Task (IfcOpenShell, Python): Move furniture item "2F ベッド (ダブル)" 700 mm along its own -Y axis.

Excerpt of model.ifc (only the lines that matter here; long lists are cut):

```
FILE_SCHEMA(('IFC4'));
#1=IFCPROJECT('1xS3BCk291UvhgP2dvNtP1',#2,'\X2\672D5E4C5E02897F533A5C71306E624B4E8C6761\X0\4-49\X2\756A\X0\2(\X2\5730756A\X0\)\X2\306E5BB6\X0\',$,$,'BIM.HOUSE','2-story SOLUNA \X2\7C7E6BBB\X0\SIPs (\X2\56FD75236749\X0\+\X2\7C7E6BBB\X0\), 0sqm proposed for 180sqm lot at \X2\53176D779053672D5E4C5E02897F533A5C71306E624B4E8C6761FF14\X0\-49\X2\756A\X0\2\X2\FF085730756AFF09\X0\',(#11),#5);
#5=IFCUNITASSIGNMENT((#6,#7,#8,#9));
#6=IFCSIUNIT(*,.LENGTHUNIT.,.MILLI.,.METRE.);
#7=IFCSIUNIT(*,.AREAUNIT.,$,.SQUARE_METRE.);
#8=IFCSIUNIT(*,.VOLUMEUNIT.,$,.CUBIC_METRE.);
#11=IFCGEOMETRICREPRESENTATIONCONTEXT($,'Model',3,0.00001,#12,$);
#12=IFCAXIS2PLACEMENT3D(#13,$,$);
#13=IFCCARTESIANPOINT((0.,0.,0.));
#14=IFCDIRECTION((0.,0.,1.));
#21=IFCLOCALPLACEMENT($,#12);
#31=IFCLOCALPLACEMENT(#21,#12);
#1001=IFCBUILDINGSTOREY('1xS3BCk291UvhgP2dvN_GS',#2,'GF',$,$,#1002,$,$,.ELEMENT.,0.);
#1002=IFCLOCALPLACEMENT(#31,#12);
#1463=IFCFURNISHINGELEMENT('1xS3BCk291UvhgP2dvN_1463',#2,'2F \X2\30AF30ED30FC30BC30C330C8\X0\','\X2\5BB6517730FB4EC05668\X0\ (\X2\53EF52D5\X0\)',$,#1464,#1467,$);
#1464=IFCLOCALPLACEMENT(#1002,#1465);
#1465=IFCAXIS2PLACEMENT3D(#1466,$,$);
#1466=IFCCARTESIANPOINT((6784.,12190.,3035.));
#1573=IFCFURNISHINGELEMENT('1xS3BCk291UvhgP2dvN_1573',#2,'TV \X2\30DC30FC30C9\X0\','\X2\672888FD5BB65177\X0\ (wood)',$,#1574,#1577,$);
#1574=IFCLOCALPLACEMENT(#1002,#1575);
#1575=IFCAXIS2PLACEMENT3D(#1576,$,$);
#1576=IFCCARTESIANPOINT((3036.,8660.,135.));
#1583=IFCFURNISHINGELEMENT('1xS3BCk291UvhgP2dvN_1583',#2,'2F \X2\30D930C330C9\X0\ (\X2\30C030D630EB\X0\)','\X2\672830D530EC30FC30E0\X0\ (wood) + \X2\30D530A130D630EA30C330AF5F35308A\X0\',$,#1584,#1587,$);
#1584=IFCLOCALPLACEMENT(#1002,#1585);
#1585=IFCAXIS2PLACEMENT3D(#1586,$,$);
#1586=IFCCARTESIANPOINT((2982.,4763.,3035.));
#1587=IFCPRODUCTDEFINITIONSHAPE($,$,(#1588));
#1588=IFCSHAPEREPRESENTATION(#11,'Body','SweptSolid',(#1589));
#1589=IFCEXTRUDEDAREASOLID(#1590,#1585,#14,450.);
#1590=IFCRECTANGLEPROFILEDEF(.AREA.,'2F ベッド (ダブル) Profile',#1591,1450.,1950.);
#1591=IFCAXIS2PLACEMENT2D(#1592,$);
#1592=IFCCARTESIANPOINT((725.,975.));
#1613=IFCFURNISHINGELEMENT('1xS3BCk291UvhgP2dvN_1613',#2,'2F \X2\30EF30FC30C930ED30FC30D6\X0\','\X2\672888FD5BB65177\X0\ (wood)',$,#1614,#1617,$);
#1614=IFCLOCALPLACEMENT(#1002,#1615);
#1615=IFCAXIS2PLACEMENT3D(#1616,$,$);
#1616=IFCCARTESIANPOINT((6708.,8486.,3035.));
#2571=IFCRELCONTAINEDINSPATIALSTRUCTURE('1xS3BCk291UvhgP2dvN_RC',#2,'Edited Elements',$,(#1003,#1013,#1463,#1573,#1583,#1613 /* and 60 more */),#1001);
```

```python
import ifcopenshell
import ifcopenshell.api.geometry
import ifcopenshell.util.placement
import ifcopenshell.util.unit

model = ifcopenshell.open("model.ifc")
unit_scale = ifcopenshell.util.unit.calculate_unit_scale(model)

item = model.by_id(1583)
matrix = ifcopenshell.util.placement.get_local_placement(item.ObjectPlacement)
matrix[:3, 3] -= matrix[:3, 1] * 0.7 / unit_scale
ifcopenshell.api.geometry.edit_object_placement(model, product=item, matrix=matrix, is_si=False)

print(ifcopenshell.util.placement.get_local_placement(item.ObjectPlacement).round(3) + 0.0)

model.write("model_updated.ifc")
```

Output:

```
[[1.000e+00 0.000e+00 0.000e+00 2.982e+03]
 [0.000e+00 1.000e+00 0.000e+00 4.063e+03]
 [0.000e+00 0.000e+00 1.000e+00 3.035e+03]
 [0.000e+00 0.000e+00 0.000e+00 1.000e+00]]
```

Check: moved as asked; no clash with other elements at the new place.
